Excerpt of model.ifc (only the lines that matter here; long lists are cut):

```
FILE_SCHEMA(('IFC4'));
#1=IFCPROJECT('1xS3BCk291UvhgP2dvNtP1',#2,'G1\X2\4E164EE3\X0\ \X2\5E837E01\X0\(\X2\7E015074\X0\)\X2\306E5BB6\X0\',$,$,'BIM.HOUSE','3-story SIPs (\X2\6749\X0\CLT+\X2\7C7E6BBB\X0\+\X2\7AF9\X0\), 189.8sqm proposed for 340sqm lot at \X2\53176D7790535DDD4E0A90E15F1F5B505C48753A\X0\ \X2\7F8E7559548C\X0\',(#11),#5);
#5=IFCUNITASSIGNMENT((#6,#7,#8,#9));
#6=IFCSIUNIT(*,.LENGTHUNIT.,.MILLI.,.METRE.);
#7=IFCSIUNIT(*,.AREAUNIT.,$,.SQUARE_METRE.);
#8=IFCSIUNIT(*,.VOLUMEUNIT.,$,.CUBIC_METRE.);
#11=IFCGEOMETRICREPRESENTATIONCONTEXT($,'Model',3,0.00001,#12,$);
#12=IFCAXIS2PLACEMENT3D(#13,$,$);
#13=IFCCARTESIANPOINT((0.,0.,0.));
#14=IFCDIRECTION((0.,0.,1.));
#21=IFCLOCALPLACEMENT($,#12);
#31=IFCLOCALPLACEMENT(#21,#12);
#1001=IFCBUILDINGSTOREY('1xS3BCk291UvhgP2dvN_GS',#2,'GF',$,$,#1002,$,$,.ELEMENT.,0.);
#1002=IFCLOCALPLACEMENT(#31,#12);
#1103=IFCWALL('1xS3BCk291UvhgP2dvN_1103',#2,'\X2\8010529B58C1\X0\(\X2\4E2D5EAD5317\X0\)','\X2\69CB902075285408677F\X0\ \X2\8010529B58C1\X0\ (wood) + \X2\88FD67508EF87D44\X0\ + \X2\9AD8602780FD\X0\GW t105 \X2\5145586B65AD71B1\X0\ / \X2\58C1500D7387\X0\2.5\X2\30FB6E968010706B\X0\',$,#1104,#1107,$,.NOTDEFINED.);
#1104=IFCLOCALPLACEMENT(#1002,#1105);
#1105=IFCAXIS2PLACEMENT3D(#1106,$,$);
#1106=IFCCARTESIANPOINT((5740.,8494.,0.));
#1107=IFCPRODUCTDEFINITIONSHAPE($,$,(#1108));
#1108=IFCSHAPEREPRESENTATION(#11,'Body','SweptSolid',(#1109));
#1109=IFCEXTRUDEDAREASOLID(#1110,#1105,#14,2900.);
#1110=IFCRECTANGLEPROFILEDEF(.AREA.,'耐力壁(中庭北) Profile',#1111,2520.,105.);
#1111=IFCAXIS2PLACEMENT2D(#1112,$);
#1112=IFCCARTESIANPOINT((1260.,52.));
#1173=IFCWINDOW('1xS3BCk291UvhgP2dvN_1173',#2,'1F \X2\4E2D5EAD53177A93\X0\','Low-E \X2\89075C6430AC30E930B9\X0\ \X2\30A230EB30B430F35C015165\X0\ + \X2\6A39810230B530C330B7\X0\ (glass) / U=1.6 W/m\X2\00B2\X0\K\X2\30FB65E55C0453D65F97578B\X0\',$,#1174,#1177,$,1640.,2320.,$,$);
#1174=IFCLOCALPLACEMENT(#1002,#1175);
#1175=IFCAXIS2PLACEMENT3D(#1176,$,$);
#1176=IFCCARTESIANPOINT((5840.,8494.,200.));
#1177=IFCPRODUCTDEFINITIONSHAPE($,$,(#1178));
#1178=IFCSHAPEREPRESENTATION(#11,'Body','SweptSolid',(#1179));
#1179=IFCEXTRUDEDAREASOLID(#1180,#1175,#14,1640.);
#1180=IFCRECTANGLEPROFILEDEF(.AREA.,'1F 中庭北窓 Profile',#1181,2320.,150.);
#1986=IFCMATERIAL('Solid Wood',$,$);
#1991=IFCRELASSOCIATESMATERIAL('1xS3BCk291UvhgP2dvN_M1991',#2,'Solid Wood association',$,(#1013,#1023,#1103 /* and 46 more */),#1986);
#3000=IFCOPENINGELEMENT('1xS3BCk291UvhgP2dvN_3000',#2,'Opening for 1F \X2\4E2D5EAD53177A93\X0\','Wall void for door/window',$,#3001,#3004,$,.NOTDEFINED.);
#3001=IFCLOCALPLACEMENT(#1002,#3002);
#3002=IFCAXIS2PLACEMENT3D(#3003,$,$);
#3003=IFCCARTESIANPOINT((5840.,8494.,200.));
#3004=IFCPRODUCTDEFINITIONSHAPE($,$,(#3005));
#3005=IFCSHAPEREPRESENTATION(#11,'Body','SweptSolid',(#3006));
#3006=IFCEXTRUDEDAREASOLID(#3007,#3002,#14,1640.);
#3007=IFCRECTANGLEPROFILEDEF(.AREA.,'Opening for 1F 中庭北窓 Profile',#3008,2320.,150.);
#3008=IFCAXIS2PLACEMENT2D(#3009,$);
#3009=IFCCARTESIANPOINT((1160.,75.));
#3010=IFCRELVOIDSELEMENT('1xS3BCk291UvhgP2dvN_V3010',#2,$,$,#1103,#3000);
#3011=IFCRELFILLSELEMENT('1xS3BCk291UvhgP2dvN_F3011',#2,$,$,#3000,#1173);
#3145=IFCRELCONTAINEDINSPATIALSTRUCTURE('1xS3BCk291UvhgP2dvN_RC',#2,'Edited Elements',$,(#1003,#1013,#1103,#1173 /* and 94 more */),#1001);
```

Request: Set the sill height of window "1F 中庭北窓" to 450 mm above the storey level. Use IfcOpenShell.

```python
import numpy as np
import ifcopenshell
import ifcopenshell.api.geometry
import ifcopenshell.geom
import ifcopenshell.util.element
import ifcopenshell.util.placement
import ifcopenshell.util.shape
import ifcopenshell.util.unit

model = ifcopenshell.open("model.ifc")
unit_scale = ifcopenshell.util.unit.calculate_unit_scale(model)

window = model.by_guid("1xS3BCk291UvhgP2dvN_1173")
opening = window.FillsVoids[0].RelatingOpeningElement
storey = ifcopenshell.util.element.get_container(window, ifc_class="IfcBuildingStorey")
level = ifcopenshell.util.placement.get_local_placement(storey.ObjectPlacement)[2, 3]

# The opening's origin need not be at the sill, so measure its lowest point.
shape = ifcopenshell.geom.create_shape(ifcopenshell.geom.settings(), opening)
bottom = ifcopenshell.util.shape.get_shape_bottom_elevation(shape, shape.geometry) / unit_scale
dz = level + 450.0 - bottom

shift = np.array([0.0, 0.0, dz])
# The window is not placed relative to its opening, so move both.
for product in (opening, window):
    matrix = ifcopenshell.util.placement.get_local_placement(product.ObjectPlacement)
    matrix[:3, 3] += shift
    ifcopenshell.api.geometry.edit_object_placement(model, product=product, matrix=matrix, is_si=False)

print(f"moved by {dz * unit_scale:+.3f} m")

model.write("model-out.ifc")
```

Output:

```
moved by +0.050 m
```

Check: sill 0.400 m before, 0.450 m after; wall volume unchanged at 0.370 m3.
